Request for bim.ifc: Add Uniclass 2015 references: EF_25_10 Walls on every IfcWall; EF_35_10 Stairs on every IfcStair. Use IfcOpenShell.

First a look at what the model holds.

```python
import ifcopenshell

model = ifcopenshell.open("bim.ifc")
print(model.schema)
print("classifications:", [c.Name for c in model.by_type("IfcClassification")])
for ifc_class in ("IfcDoor", "IfcRoof", "IfcStair", "IfcWall", "IfcWindow"):
    print(ifc_class, len(model.by_type(ifc_class)))
```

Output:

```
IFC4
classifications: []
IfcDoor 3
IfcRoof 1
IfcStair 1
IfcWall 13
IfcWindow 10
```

```python
import ifcopenshell
import ifcopenshell.api.classification

model = ifcopenshell.open("bim.ifc")

system = ifcopenshell.api.classification.add_classification(model, classification="Uniclass 2015")

codes = {
    "IfcWall": ("EF_25_10", "Walls"),
    "IfcStair": ("EF_35_10", "Stairs"),
}
for ifc_class, (code, name) in codes.items():
    products = model.by_type(ifc_class)
    ifcopenshell.api.classification.add_reference(
        model, products=products, classification=system, identification=code, name=name
    )
    print(code, len(products))

model.write("bim_updated.ifc")
```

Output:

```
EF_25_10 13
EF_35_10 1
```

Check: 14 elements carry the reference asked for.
